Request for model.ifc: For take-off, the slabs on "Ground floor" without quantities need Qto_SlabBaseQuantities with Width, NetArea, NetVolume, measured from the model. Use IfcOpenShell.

First a look at what the model holds.

```python
import ifcopenshell
import ifcopenshell.util.element
import ifcopenshell.util.unit

model = ifcopenshell.open("model.ifc")
print(model.schema)
for unit_type in ("LENGTHUNIT", "AREAUNIT", "VOLUMEUNIT"):
    print(unit_type, ifcopenshell.util.unit.calculate_unit_scale(model, unit_type))
storey = next(s for s in model.by_type("IfcBuildingStorey") if s.Name == "Ground floor")
slabs = [e for e in ifcopenshell.util.element.get_decomposition(storey) if e.is_a("IfcSlab")]
for e in sorted(slabs, key=lambda e: e.id()):
    print(e.id(), e.is_a(), e.Name, list(ifcopenshell.util.element.get_psets(e, qtos_only=True)), sep=" | ")
```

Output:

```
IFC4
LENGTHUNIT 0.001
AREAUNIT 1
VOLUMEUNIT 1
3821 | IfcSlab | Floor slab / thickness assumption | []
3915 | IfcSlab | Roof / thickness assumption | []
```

```python
import ifcopenshell
import ifcopenshell.api.pset
import ifcopenshell.geom
import ifcopenshell.util.element
import ifcopenshell.util.shape
import ifcopenshell.util.unit

model = ifcopenshell.open("model.ifc")
unit_scale = ifcopenshell.util.unit.calculate_unit_scale(model)
area_scale = ifcopenshell.util.unit.calculate_unit_scale(model, "AREAUNIT")
volume_scale = ifcopenshell.util.unit.calculate_unit_scale(model, "VOLUMEUNIT")
settings = ifcopenshell.geom.settings()

storey = next(s for s in model.by_type("IfcBuildingStorey") if s.Name == "Ground floor")
slabs = [e for e in ifcopenshell.util.element.get_decomposition(storey) if e.is_a("IfcSlab")]

for e in sorted(slabs, key=lambda e: e.id()):
    if ifcopenshell.util.element.get_psets(e, qtos_only=True, should_inherit=False):
        continue
    # Geometry comes back in metres, in the element's own axes.
    shape = ifcopenshell.geom.create_shape(settings, e)
    values = {
        "Width": ifcopenshell.util.shape.get_z(shape.geometry) / unit_scale,
        "NetArea": ifcopenshell.util.shape.get_footprint_area(shape.geometry) / area_scale,
        "NetVolume": ifcopenshell.util.shape.get_volume(shape.geometry) / volume_scale,
    }
    qto = ifcopenshell.api.pset.add_qto(model, product=e, name="Qto_SlabBaseQuantities")
    ifcopenshell.api.pset.edit_qto(model, qto=qto, properties=values)
    print(e.id(), {k: round(v, 3) for k, v in values.items()})

model.write("model_edited.ifc")
```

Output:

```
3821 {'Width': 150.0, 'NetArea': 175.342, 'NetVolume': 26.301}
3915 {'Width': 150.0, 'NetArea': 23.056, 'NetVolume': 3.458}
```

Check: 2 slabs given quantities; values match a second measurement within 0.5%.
